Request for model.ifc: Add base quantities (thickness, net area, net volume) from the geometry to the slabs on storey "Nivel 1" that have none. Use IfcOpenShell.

First a look at what the model holds.

```python
import ifcopenshell
import ifcopenshell.util.element
import ifcopenshell.util.unit

model = ifcopenshell.open("model.ifc")
print(model.schema)
for unit_type in ("LENGTHUNIT", "AREAUNIT", "VOLUMEUNIT"):
    print(unit_type, ifcopenshell.util.unit.calculate_unit_scale(model, unit_type))
storey = next(s for s in model.by_type("IfcBuildingStorey") if s.Name == "Nivel 1")
slabs = [e for e in ifcopenshell.util.element.get_decomposition(storey) if e.is_a("IfcSlab")]
for e in sorted(slabs, key=lambda e: e.id()):
    print(e.id(), e.is_a(), e.Name, list(ifcopenshell.util.element.get_psets(e, qtos_only=True)), sep=" | ")
```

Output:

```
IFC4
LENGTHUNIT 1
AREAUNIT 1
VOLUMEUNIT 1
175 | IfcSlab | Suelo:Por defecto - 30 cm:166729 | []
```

```python
import ifcopenshell
import ifcopenshell.api.pset
import ifcopenshell.geom
import ifcopenshell.util.element
import ifcopenshell.util.shape
import ifcopenshell.util.unit

model = ifcopenshell.open("model.ifc")
unit_scale = ifcopenshell.util.unit.calculate_unit_scale(model)
area_scale = ifcopenshell.util.unit.calculate_unit_scale(model, "AREAUNIT")
volume_scale = ifcopenshell.util.unit.calculate_unit_scale(model, "VOLUMEUNIT")
settings = ifcopenshell.geom.settings()

storey = next(s for s in model.by_type("IfcBuildingStorey") if s.Name == "Nivel 1")
slabs = [e for e in ifcopenshell.util.element.get_decomposition(storey) if e.is_a("IfcSlab")]

for e in sorted(slabs, key=lambda e: e.id()):
    if ifcopenshell.util.element.get_psets(e, qtos_only=True, should_inherit=False):
        continue
    # Geometry comes back in metres, in the element's own axes.
    shape = ifcopenshell.geom.create_shape(settings, e)
    values = {
        "Width": ifcopenshell.util.shape.get_z(shape.geometry) / unit_scale,
        "NetArea": ifcopenshell.util.shape.get_footprint_area(shape.geometry) / area_scale,
        "NetVolume": ifcopenshell.util.shape.get_volume(shape.geometry) / volume_scale,
    }
    qto = ifcopenshell.api.pset.add_qto(model, product=e, name="Qto_SlabBaseQuantities")
    ifcopenshell.api.pset.edit_qto(model, qto=qto, properties=values)
    print(e.id(), {k: round(v, 3) for k, v in values.items()})

model.write("model_v2.ifc")
```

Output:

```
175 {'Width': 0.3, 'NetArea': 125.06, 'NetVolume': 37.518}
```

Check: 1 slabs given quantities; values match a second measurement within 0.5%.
